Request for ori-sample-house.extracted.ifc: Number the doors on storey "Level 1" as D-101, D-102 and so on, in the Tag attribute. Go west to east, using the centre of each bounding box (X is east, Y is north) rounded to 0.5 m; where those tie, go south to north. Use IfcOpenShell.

First a look at what the model holds.

```python
import ifcopenshell
import ifcopenshell.util.element
import ifcopenshell.util.placement

model = ifcopenshell.open("ori-sample-house.extracted.ifc")
print(model.schema)
storey = next(s for s in model.by_type("IfcBuildingStorey") if s.Name == "Level 1")
doors = [e for e in ifcopenshell.util.element.get_decomposition(storey) if e.is_a("IfcDoor")]
for e in sorted(doors, key=lambda e: e.id()):
    origin = ifcopenshell.util.placement.get_local_placement(e.ObjectPlacement)[:3, 3]
    print(e.id(), e.Tag, e.Name, origin.round(2) + 0.0, sep=" | ")
```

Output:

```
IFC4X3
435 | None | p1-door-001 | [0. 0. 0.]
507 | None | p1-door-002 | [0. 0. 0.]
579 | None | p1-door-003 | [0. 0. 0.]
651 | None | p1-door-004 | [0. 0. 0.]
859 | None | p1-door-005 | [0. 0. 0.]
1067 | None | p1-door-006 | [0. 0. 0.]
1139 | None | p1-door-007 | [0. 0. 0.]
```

```python
import ifcopenshell
import ifcopenshell.geom
import ifcopenshell.util.element
import ifcopenshell.util.shape

model = ifcopenshell.open("ori-sample-house.extracted.ifc")
settings = ifcopenshell.geom.settings()
settings.set("use-world-coords", True)


def centre(element):
    shape = ifcopenshell.geom.create_shape(settings, element)
    return ifcopenshell.util.shape.get_bbox_centroid(shape.geometry)


storey = next(s for s in model.by_type("IfcBuildingStorey") if s.Name == "Level 1")
doors = [e for e in ifcopenshell.util.element.get_decomposition(storey) if e.is_a("IfcDoor")]

# Insertion points can sit at a corner or the storey origin, so sort by the geometry (in metres).
centres = {e: centre(e) for e in doors}
doors.sort(key=lambda e: (round(centres[e][0] / 0.5), centres[e][1]))

for i, e in enumerate(doors, start=1):
    number = f"D-1{i:02d}"
    e.Tag = number
    print(e.id(), number)

model.write("ori-sample-house.extracted_v2.ifc")
```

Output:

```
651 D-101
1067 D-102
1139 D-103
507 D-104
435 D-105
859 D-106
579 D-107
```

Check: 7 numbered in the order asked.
